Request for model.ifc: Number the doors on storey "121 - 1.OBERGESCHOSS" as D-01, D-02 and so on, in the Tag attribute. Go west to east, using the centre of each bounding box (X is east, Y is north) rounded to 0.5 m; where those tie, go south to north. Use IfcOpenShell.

First a look at what the model holds.

```python
import ifcopenshell
import ifcopenshell.util.element
import ifcopenshell.util.placement

model = ifcopenshell.open("model.ifc")
print(model.schema)
storey = next(s for s in model.by_type("IfcBuildingStorey") if s.Name == "121 - 1.OBERGESCHOSS")
doors = [e for e in ifcopenshell.util.element.get_decomposition(storey) if e.is_a("IfcDoor")]
for e in sorted(doors, key=lambda e: e.id()):
    origin = ifcopenshell.util.placement.get_local_placement(e.ObjectPlacement)[:3, 3]
    print(e.id(), e.Tag, e.Name, origin.round(2) + 0.0, sep=" | ")
```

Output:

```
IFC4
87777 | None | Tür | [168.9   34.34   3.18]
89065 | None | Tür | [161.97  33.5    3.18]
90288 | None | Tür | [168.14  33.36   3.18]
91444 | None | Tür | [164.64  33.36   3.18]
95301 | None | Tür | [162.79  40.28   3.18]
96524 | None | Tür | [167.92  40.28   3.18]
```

```python
import ifcopenshell
import ifcopenshell.geom
import ifcopenshell.util.element
import ifcopenshell.util.shape

model = ifcopenshell.open("model.ifc")
settings = ifcopenshell.geom.settings()
settings.set("use-world-coords", True)


def centre(element):
    shape = ifcopenshell.geom.create_shape(settings, element)
    return ifcopenshell.util.shape.get_bbox_centroid(shape.geometry)


storey = next(s for s in model.by_type("IfcBuildingStorey") if s.Name == "121 - 1.OBERGESCHOSS")
doors = [e for e in ifcopenshell.util.element.get_decomposition(storey) if e.is_a("IfcDoor")]

# Insertion points can sit at a corner or the storey origin, so sort by the geometry (in metres).
centres = {e: centre(e) for e in doors}
doors.sort(key=lambda e: (round(centres[e][0] / 0.5), centres[e][1]))

for i, e in enumerate(doors, start=1):
    number = f"D-{i:02d}"
    e.Tag = number
    print(e.id(), number)

model.write("model_updated.ifc")
```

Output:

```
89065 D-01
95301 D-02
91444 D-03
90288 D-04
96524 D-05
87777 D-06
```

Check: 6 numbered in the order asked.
